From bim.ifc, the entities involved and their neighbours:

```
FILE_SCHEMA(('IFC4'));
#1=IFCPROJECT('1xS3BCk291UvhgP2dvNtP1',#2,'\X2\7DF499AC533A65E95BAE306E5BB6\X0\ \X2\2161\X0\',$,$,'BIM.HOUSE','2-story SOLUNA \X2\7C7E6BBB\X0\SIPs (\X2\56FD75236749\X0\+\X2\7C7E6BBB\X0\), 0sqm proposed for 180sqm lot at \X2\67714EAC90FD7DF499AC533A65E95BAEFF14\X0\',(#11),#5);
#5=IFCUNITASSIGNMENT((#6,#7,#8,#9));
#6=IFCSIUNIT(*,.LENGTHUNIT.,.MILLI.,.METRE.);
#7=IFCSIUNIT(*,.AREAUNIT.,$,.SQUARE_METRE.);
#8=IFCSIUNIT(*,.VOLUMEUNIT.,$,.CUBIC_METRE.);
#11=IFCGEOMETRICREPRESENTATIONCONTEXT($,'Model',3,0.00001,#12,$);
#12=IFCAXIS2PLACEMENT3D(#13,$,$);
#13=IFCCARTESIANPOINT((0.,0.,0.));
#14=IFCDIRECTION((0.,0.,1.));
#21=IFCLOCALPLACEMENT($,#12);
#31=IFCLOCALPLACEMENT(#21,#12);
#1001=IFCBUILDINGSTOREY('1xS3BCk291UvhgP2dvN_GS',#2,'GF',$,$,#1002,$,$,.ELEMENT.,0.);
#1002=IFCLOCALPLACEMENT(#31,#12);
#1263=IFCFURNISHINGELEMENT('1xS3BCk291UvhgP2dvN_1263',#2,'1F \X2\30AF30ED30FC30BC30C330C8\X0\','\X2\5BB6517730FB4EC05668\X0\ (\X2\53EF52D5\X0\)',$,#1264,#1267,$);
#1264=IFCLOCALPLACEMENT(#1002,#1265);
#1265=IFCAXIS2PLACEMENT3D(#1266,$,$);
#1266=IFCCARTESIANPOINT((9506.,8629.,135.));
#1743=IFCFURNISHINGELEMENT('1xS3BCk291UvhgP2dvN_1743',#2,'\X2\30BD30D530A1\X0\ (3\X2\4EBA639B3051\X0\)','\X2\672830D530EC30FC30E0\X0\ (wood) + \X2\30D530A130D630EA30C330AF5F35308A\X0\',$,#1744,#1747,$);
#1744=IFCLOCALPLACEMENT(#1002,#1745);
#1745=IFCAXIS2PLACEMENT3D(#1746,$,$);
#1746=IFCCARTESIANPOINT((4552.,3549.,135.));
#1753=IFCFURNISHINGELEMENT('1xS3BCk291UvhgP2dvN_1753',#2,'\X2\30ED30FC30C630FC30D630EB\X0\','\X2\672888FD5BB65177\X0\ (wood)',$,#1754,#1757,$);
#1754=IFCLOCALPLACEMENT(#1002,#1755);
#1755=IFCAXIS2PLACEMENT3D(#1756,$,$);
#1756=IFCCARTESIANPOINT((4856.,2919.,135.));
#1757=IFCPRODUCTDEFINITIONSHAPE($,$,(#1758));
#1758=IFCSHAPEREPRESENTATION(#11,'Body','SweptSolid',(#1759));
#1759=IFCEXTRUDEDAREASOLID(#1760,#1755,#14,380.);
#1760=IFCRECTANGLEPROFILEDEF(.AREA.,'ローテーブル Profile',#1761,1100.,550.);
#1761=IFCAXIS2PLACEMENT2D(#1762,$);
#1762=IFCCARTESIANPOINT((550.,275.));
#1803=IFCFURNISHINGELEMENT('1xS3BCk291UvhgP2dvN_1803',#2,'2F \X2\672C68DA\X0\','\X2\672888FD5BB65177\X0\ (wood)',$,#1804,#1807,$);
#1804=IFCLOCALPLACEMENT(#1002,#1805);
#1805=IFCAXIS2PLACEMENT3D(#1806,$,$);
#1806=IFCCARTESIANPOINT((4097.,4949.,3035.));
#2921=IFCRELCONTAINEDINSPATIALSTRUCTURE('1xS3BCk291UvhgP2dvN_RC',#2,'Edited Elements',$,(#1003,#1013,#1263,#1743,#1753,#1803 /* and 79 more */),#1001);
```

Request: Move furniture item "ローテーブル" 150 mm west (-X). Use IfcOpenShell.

```python
import ifcopenshell
import ifcopenshell.api.geometry
import ifcopenshell.util.placement
import ifcopenshell.util.unit

model = ifcopenshell.open("bim.ifc")
unit_scale = ifcopenshell.util.unit.calculate_unit_scale(model)

item = model.by_guid("1xS3BCk291UvhgP2dvN_1753")
matrix = ifcopenshell.util.placement.get_local_placement(item.ObjectPlacement)
matrix[0, 3] -= 0.15 / unit_scale
ifcopenshell.api.geometry.edit_object_placement(model, product=item, matrix=matrix, is_si=False)

print(ifcopenshell.util.placement.get_local_placement(item.ObjectPlacement).round(3) + 0.0)

model.write("bim_edited.ifc")
```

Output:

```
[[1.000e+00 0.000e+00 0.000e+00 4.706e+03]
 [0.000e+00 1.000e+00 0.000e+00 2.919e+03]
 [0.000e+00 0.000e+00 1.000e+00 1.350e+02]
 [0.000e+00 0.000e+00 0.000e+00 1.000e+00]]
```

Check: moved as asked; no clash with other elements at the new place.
